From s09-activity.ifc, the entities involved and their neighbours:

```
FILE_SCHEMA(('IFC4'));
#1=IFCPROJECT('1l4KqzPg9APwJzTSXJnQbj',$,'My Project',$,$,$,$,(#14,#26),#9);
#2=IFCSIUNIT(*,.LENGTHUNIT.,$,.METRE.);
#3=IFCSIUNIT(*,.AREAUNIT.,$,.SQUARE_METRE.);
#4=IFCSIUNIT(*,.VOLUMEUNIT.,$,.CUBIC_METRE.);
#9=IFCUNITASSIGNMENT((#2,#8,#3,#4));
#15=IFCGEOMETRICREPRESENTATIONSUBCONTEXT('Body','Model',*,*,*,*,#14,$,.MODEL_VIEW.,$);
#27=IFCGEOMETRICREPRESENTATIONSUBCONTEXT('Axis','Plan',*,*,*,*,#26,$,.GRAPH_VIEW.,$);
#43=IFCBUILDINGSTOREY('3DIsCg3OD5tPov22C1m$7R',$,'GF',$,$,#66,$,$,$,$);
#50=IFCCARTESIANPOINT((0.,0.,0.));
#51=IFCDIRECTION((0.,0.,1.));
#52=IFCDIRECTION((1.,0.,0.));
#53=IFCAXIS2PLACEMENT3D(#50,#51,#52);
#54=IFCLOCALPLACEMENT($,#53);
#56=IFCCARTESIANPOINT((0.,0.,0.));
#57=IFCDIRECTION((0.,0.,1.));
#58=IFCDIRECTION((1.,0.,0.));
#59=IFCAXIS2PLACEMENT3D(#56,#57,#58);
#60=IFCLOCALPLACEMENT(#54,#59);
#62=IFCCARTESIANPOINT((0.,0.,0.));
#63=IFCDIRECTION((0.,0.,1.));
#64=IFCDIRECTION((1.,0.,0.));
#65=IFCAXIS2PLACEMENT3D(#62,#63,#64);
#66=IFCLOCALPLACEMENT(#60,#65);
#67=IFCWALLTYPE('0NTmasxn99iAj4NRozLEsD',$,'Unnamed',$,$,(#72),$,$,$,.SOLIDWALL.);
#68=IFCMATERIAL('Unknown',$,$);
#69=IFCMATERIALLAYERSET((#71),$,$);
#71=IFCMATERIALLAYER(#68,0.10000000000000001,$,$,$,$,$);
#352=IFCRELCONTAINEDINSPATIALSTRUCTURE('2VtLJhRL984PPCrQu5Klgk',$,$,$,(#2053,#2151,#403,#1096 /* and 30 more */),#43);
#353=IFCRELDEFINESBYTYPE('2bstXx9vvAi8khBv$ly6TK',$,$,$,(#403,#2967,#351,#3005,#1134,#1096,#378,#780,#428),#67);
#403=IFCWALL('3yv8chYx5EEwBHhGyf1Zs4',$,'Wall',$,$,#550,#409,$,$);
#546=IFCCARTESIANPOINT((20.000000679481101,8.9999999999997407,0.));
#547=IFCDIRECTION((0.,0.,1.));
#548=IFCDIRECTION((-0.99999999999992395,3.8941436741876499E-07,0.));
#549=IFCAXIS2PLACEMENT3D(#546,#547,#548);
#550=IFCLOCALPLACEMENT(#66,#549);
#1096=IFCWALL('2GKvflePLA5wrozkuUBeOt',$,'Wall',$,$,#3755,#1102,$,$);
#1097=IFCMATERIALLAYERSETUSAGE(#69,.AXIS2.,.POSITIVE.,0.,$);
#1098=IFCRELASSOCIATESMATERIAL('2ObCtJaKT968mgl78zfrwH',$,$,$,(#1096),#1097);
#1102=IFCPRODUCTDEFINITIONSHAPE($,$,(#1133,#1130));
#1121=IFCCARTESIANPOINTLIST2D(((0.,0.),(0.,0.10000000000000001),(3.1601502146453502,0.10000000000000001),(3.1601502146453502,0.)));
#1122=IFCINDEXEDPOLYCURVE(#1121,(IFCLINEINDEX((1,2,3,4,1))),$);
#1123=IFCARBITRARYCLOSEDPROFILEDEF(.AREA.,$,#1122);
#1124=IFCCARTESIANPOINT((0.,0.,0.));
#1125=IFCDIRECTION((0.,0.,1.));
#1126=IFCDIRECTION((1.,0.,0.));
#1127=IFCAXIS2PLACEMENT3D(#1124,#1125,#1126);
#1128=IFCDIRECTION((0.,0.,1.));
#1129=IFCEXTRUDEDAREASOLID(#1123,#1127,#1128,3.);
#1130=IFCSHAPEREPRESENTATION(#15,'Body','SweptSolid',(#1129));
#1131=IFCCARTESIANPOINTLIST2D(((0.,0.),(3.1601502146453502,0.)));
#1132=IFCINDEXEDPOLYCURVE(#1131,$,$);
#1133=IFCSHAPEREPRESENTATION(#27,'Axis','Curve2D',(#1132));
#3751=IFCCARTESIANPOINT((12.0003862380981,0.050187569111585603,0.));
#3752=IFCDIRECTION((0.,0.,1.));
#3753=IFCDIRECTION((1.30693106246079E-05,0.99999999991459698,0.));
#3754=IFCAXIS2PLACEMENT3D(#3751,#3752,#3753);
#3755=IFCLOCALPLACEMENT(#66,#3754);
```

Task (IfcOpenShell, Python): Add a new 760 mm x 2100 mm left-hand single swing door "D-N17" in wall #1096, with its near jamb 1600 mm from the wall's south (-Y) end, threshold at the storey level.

```python
import numpy as np
import ifcopenshell
import ifcopenshell.api.feature
import ifcopenshell.api.geometry
import ifcopenshell.api.root
import ifcopenshell.api.spatial
import ifcopenshell.geom
import ifcopenshell.util.element
import ifcopenshell.util.placement
import ifcopenshell.util.representation
import ifcopenshell.util.shape
import ifcopenshell.util.unit

model = ifcopenshell.open("s09-activity.ifc")
unit_scale = ifcopenshell.util.unit.calculate_unit_scale(model)
settings = ifcopenshell.geom.settings()


def volume(element):
    """Net volume in cubic metres, openings subtracted."""
    shape = ifcopenshell.geom.create_shape(settings, element)
    return ifcopenshell.util.shape.get_volume(shape.geometry)


wall = model.by_guid("2GKvflePLA5wrozkuUBeOt")
storey = ifcopenshell.util.element.get_container(wall, ifc_class="IfcBuildingStorey")
context = ifcopenshell.util.representation.get_context(model, "Model", "Body", "MODEL_VIEW")
before = volume(wall)

width, height, from_end, sill = 0.76, 2.1, 1.6, 0.0  # metres

# The wall runs along its own X axis, and the end named is its -X end.
wall_shape = ifcopenshell.geom.create_shape(settings, wall)
x, y, z = ifcopenshell.util.shape.get_vertices(wall_shape.geometry).T
start = x.min() + from_end
face, thickness = float(y.min()), float(y.max() - y.min())
wall_matrix = ifcopenshell.util.placement.get_local_placement(wall.ObjectPlacement)
level = ifcopenshell.util.placement.get_local_placement(storey.ObjectPlacement)[2, 3]


def in_wall(x, y):
    """Placement at x, y metres in the wall's axes, at sill height."""
    matrix = wall_matrix.copy()
    matrix[:, 3] = wall_matrix @ np.array([x / unit_scale, y / unit_scale, 0.0, 1.0])
    matrix[2, 3] = level + sill / unit_scale
    return matrix


# Opening: a box that overshoots both wall faces by 50 mm.
opening = ifcopenshell.api.root.create_entity(model, ifc_class="IfcOpeningElement", predefined_type="OPENING")
box = ifcopenshell.api.geometry.add_wall_representation(
    model, context=context, length=width, height=height, thickness=thickness + 0.1
)
ifcopenshell.api.geometry.assign_representation(model, product=opening, representation=box)
ifcopenshell.api.geometry.edit_object_placement(model, product=opening, matrix=in_wall(start, face - 0.05), is_si=False)
ifcopenshell.api.feature.add_feature(model, feature=opening, element=wall)

door = ifcopenshell.api.root.create_entity(model, ifc_class="IfcDoor", name="D-N17", predefined_type="DOOR")
door.OverallWidth, door.OverallHeight = width / unit_scale, height / unit_scale
door.OperationType = "SINGLE_SWING_LEFT"
body = ifcopenshell.api.geometry.add_door_representation(
    model,
    context=context,
    overall_width=door.OverallWidth,
    overall_height=door.OverallHeight,
    operation_type="SINGLE_SWING_LEFT",
    lining_properties={"LiningDepth": thickness / unit_scale, "ThresholdDepth": thickness / unit_scale},
)
ifcopenshell.api.geometry.assign_representation(model, product=door, representation=body)
ifcopenshell.api.spatial.assign_container(model, products=[door], relating_structure=storey)
ifcopenshell.api.feature.add_filling(model, opening=opening, element=door)

# The lining spans the wall, so the door starts at the wall face.
ifcopenshell.api.geometry.edit_object_placement(model, product=door, matrix=in_wall(start, face), is_si=False)

after = volume(wall)

print(f"wall volume {before:.3f} -> {after:.3f} m3")

model.write("s09-activity_rev.ifc")
```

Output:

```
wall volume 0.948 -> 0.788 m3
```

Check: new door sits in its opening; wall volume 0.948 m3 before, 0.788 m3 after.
